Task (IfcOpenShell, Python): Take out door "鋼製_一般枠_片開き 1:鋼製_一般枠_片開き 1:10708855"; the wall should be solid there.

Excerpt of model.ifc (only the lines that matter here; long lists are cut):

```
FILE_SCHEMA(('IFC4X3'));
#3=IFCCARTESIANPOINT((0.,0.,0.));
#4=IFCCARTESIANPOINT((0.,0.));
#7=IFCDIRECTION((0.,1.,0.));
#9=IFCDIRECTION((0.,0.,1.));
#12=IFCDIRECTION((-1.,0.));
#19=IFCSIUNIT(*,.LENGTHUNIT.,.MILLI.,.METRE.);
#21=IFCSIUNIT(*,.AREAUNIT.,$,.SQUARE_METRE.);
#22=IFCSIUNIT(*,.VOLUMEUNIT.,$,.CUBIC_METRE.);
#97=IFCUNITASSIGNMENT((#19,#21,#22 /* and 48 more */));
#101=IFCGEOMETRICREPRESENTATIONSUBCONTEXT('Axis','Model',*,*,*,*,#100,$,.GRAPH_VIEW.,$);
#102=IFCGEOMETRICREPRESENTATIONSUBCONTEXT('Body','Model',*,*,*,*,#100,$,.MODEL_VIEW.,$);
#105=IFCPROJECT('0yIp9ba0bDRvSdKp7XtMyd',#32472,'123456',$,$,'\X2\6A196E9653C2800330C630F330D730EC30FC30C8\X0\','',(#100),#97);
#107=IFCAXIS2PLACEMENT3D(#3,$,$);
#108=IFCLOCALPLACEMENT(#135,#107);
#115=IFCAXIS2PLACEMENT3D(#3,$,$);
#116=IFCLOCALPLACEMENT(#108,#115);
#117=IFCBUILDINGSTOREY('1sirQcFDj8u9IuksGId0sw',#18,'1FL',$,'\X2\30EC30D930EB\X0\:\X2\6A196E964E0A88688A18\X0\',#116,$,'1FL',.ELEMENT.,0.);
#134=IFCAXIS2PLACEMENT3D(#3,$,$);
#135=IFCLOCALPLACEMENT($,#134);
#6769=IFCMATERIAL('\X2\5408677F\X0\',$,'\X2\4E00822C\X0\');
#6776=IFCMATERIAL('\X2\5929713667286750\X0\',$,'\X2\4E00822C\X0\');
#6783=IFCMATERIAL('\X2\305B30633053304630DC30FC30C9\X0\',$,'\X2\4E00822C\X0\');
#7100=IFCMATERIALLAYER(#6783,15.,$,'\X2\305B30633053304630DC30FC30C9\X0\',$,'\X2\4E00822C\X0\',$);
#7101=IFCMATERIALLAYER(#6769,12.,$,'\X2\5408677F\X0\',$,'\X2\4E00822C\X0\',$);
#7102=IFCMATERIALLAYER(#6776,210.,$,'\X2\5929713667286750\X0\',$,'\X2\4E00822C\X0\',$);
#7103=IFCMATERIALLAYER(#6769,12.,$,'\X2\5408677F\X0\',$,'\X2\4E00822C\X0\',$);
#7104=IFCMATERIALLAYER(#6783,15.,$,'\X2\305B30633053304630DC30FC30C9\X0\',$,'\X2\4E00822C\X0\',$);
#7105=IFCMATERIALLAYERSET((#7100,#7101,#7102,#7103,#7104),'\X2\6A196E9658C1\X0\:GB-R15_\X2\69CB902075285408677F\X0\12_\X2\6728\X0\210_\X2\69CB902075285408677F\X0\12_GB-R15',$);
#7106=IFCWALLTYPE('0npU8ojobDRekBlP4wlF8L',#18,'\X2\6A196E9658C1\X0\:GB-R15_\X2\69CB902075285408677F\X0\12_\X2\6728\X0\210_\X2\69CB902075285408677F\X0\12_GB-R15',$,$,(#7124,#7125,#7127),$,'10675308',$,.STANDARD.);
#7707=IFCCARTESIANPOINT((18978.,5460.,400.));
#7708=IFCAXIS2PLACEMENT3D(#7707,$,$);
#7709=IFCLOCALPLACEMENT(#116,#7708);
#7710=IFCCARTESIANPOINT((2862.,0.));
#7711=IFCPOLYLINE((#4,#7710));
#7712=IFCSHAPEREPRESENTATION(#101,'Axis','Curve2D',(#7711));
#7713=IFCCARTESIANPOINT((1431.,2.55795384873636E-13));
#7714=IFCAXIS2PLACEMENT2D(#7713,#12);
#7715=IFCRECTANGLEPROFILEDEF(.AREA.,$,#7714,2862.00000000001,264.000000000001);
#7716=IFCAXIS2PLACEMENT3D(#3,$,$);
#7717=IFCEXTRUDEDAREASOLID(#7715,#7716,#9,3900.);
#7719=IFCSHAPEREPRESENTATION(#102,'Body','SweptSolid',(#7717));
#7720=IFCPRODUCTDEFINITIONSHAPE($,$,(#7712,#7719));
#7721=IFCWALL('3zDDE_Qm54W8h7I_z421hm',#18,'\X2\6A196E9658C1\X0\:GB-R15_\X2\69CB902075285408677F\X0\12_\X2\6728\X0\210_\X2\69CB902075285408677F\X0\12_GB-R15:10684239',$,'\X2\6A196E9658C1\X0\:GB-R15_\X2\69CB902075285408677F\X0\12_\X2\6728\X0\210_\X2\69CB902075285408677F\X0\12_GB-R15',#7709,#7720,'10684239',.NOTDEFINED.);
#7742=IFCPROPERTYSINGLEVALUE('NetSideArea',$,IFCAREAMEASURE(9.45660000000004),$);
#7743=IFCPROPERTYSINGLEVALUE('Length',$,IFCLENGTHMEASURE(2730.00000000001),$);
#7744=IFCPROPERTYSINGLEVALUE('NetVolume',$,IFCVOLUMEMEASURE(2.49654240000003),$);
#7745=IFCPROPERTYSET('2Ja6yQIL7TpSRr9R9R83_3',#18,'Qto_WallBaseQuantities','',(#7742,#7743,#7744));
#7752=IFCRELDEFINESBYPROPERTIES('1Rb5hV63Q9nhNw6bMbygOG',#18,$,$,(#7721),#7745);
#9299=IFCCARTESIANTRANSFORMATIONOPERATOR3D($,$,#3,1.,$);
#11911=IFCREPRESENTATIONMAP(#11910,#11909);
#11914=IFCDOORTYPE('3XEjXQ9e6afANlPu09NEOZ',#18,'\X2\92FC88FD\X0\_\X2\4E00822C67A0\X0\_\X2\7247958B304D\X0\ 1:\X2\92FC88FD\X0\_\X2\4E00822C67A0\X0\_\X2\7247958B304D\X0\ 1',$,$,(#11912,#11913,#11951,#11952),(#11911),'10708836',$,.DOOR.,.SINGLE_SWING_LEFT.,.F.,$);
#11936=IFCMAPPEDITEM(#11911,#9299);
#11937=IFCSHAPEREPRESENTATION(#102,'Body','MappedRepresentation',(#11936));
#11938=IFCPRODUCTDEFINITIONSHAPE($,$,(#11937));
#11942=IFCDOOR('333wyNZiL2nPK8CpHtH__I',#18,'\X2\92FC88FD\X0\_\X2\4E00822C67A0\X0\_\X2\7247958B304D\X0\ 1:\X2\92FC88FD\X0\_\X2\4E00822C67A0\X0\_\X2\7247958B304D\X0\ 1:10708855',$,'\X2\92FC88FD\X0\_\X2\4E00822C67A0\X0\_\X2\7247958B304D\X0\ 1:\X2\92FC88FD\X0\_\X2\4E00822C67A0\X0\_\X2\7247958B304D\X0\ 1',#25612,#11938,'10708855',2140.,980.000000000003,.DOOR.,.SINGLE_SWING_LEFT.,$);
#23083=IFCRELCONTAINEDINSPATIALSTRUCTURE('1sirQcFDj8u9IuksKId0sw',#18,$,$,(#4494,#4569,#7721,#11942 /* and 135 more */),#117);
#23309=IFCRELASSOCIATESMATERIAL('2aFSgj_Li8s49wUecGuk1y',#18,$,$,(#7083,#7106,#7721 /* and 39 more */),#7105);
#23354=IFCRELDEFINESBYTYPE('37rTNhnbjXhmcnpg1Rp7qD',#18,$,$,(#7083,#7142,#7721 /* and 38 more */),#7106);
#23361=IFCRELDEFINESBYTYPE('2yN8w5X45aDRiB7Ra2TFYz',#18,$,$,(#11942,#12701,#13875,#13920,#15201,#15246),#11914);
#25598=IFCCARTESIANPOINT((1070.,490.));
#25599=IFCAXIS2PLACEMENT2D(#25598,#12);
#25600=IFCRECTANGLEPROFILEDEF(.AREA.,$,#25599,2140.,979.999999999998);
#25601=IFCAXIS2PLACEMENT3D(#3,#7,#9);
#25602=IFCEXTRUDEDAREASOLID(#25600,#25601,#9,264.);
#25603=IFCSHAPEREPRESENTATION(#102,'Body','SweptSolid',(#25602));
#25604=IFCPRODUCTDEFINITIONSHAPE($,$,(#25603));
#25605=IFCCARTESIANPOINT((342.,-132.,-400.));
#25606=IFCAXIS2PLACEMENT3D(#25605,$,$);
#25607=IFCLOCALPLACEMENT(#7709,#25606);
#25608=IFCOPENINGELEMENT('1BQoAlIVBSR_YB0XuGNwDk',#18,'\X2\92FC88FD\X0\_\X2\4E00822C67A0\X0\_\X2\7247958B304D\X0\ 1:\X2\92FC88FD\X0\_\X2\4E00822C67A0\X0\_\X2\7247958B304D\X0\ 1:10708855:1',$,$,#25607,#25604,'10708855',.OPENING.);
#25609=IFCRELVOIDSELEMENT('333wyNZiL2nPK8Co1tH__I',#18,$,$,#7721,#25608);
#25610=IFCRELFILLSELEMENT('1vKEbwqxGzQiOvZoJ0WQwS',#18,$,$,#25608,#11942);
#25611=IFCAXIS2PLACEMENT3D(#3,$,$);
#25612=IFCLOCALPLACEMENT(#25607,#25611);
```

```python
import ifcopenshell
import ifcopenshell.api.feature
import ifcopenshell.api.pset
import ifcopenshell.api.root
import ifcopenshell.geom
import ifcopenshell.util.element
import ifcopenshell.util.shape
import ifcopenshell.util.unit

model = ifcopenshell.open("model.ifc")
area_scale = ifcopenshell.util.unit.calculate_unit_scale(model, "AREAUNIT")
volume_scale = ifcopenshell.util.unit.calculate_unit_scale(model, "VOLUMEUNIT")
settings = ifcopenshell.geom.settings()


def volume(element):
    """Net volume in cubic metres, openings subtracted."""
    shape = ifcopenshell.geom.create_shape(settings, element)
    return ifcopenshell.util.shape.get_volume(shape.geometry)


door = model.by_id(11942)
opening = door.FillsVoids[0].RelatingOpeningElement
wall = opening.VoidsElements[0].RelatingBuildingElement
before = volume(wall)

ifcopenshell.api.root.remove_product(model, product=door)
ifcopenshell.api.feature.remove_feature(model, feature=opening)

after = volume(wall)
thickness = 0.264  # wall thickness in metres

# Update the wall's stored quantities.
pset = model.by_id(ifcopenshell.util.element.get_pset(wall, "Qto_WallBaseQuantities", should_inherit=False)["id"])
ifcopenshell.api.pset.edit_pset(model, pset=pset, properties={
    "NetSideArea": model.create_entity("IfcAreaMeasure", after / thickness / area_scale),
    "NetVolume": model.create_entity("IfcVolumeMeasure", after / volume_scale),
})

print(f"wall volume {before:.3f} -> {after:.3f} m3")

model.write("model_rev.ifc")
```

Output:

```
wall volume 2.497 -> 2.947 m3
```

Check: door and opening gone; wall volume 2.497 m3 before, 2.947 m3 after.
